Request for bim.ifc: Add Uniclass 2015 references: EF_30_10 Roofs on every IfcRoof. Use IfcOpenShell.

First a look at what the model holds.

```python
import ifcopenshell

model = ifcopenshell.open("bim.ifc")
print(model.schema)
print("classifications:", [c.Name for c in model.by_type("IfcClassification")])
for ifc_class in ("IfcDoor", "IfcRoof", "IfcStair", "IfcWall", "IfcWindow"):
    print(ifc_class, len(model.by_type(ifc_class)))
```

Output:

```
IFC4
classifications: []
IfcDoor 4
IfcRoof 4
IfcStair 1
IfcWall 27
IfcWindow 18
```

```python
import ifcopenshell
import ifcopenshell.api.classification

model = ifcopenshell.open("bim.ifc")

system = ifcopenshell.api.classification.add_classification(model, classification="Uniclass 2015")

codes = {
    "IfcRoof": ("EF_30_10", "Roofs"),
}
for ifc_class, (code, name) in codes.items():
    products = model.by_type(ifc_class)
    ifcopenshell.api.classification.add_reference(
        model, products=products, classification=system, identification=code, name=name
    )
    print(code, len(products))

model.write("bim_updated.ifc")
```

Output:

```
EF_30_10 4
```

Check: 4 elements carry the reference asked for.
